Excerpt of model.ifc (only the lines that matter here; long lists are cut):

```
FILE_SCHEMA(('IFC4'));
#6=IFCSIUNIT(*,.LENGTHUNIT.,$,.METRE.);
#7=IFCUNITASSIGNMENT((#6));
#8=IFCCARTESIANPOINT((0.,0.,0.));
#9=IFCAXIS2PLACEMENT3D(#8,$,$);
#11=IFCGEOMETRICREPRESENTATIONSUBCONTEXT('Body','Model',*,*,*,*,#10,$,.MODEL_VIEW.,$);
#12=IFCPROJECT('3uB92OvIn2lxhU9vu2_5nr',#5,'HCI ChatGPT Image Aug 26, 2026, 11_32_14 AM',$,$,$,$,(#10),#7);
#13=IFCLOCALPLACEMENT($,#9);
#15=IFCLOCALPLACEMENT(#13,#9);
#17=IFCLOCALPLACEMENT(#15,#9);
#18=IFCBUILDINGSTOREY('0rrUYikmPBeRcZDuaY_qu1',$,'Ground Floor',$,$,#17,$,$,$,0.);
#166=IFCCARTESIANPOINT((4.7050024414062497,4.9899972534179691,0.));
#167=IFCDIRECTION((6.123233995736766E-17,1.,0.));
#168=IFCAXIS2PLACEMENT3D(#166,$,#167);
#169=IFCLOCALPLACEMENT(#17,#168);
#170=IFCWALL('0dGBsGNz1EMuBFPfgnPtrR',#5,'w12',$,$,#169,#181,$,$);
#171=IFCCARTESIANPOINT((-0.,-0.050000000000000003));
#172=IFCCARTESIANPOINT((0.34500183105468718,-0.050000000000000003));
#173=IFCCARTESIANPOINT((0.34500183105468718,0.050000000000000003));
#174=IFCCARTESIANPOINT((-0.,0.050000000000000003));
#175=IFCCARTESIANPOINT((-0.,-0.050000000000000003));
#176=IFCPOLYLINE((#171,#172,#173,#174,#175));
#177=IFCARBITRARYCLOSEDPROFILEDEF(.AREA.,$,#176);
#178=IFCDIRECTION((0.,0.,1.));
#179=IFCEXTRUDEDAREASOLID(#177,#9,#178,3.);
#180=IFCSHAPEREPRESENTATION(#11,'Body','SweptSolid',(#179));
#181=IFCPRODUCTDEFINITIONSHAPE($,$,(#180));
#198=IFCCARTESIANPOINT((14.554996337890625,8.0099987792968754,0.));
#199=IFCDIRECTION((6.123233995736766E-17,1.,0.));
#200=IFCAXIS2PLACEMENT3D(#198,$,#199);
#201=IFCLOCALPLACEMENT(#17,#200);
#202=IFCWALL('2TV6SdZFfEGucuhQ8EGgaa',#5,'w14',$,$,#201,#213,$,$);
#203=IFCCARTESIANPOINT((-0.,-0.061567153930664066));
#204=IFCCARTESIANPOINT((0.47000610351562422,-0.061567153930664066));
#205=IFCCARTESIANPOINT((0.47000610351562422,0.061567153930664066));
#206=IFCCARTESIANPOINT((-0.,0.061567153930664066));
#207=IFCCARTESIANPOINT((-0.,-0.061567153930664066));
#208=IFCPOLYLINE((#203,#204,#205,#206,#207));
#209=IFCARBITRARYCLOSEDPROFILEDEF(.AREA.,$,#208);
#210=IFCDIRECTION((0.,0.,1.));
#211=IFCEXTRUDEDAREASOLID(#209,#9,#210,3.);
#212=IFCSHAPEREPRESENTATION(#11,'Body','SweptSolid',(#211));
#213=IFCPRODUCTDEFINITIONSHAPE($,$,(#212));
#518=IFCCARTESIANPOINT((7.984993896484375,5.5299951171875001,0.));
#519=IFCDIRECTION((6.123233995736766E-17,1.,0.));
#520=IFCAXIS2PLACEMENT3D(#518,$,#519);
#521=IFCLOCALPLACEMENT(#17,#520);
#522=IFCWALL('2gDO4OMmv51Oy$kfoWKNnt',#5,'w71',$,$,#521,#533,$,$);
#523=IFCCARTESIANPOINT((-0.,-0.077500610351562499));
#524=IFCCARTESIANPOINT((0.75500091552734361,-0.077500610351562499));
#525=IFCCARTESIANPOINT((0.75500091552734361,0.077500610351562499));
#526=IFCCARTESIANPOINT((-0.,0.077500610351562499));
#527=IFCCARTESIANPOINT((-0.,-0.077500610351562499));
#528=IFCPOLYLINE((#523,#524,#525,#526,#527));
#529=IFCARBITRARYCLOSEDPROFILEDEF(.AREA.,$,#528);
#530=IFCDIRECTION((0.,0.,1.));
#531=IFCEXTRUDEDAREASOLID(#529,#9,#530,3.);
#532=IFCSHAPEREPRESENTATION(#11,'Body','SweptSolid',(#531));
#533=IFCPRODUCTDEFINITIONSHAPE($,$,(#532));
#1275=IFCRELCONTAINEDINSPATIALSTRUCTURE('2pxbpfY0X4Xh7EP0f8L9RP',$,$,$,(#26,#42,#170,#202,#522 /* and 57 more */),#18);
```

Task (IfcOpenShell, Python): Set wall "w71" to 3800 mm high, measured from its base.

```python
import ifcopenshell
import ifcopenshell.geom
import ifcopenshell.util.representation
import ifcopenshell.util.shape
import ifcopenshell.util.unit

model = ifcopenshell.open("model.ifc")
unit_scale = ifcopenshell.util.unit.calculate_unit_scale(model)
settings = ifcopenshell.geom.settings()


def volume(element):
    """Net volume in cubic metres, openings subtracted."""
    shape = ifcopenshell.geom.create_shape(settings, element)
    return ifcopenshell.util.shape.get_volume(shape.geometry)


wall = model.by_guid("2gDO4OMmv51Oy$kfoWKNnt")
before = volume(wall)

body = ifcopenshell.util.representation.get_representation(wall, "Model", "Body")
solid = body.Items[0]
old_height = solid.Depth
solid.Depth = 3.8 / unit_scale
after = volume(wall)

print(f"height {old_height:g} -> {solid.Depth:g}, volume {before:.3f} -> {after:.3f} m3")

model.write("model_updated.ifc")
```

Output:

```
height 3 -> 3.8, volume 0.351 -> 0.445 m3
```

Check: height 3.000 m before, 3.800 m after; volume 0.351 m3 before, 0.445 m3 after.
